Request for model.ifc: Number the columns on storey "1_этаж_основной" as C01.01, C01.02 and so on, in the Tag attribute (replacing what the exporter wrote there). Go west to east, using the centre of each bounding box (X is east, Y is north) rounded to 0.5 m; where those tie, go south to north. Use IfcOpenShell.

First a look at what the model holds.

```python
import ifcopenshell
import ifcopenshell.util.element
import ifcopenshell.util.placement

model = ifcopenshell.open("model.ifc")
print(model.schema)
storey = next(s for s in model.by_type("IfcBuildingStorey") if s.Name == "1_этаж_основной")
columns = [e for e in ifcopenshell.util.element.get_decomposition(storey) if e.is_a("IfcColumn")]
for e in sorted(columns, key=lambda e: e.id()):
    origin = ifcopenshell.util.placement.get_local_placement(e.ObjectPlacement)[:3, 3]
    print(e.id(), e.Tag, e.Name, origin.round(2) + 0.0, sep=" | ")
```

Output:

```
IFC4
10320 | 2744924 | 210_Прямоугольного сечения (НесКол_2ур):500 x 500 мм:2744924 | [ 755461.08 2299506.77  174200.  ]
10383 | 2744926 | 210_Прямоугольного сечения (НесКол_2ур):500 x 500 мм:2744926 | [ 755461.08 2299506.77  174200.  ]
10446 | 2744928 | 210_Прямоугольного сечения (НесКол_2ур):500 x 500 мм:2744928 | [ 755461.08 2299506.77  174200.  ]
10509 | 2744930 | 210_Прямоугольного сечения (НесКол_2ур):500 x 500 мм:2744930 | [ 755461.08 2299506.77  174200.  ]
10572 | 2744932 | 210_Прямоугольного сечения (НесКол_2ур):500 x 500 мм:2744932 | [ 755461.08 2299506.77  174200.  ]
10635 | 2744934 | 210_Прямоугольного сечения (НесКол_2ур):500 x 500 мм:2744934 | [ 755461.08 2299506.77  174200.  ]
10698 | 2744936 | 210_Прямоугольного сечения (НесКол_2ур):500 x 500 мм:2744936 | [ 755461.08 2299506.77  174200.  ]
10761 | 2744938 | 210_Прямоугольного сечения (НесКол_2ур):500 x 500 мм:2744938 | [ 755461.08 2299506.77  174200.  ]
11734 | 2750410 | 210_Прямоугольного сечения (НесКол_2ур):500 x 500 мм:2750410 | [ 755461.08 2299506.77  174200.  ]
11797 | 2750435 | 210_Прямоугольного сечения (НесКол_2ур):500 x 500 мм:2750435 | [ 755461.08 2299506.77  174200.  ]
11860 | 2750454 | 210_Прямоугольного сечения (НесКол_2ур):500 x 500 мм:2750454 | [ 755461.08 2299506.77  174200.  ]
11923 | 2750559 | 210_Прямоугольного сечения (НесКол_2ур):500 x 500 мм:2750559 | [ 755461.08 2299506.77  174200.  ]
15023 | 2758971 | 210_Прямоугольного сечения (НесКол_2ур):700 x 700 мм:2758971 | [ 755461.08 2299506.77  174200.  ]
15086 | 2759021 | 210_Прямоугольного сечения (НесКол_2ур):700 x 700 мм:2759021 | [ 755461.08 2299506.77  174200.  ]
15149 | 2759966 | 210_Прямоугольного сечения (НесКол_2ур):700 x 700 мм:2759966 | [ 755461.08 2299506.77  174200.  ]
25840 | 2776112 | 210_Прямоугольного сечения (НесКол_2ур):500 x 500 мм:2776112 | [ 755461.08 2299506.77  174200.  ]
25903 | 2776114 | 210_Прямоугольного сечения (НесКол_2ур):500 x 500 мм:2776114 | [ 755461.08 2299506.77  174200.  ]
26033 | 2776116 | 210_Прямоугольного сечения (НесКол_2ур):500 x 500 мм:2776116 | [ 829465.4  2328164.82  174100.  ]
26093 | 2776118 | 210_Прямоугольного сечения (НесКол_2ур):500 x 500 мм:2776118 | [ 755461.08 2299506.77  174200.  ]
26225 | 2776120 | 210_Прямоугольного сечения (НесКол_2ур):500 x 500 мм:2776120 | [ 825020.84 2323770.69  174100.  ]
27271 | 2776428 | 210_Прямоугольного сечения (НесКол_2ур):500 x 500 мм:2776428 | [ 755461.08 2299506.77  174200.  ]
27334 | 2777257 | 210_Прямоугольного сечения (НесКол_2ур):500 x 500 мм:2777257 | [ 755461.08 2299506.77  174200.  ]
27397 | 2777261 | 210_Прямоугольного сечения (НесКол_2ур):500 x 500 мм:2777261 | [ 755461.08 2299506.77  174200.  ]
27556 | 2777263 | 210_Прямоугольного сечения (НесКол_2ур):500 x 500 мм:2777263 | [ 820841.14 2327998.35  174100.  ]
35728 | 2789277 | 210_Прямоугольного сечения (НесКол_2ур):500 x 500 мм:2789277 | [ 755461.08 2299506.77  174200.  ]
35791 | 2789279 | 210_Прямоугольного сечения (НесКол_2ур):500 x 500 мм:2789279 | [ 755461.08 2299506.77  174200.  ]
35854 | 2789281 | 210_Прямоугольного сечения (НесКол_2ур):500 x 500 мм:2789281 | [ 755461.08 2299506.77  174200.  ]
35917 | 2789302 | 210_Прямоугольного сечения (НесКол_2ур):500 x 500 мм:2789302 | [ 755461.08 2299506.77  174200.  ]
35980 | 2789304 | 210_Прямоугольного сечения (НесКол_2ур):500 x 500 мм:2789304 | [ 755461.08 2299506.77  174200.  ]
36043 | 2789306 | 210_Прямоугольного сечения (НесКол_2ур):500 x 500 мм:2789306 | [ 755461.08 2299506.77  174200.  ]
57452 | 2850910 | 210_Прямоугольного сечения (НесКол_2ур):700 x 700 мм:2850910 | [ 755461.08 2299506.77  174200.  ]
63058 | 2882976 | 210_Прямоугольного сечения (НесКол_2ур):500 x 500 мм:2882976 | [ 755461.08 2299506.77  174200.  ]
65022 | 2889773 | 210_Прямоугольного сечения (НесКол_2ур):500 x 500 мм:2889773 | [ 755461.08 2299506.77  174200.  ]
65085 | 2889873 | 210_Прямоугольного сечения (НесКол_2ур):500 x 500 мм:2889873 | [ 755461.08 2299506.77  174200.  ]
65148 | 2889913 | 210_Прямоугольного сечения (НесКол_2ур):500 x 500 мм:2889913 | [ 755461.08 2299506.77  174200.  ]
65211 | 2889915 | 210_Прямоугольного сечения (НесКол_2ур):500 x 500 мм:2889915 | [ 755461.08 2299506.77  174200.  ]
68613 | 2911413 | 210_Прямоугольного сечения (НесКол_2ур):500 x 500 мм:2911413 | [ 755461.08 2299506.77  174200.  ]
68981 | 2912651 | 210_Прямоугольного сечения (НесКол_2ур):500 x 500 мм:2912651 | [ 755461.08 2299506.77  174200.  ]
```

```python
import ifcopenshell
import ifcopenshell.geom
import ifcopenshell.util.element
import ifcopenshell.util.shape

model = ifcopenshell.open("model.ifc")
settings = ifcopenshell.geom.settings()
settings.set("use-world-coords", True)


def centre(element):
    shape = ifcopenshell.geom.create_shape(settings, element)
    return ifcopenshell.util.shape.get_bbox_centroid(shape.geometry)


storey = next(s for s in model.by_type("IfcBuildingStorey") if s.Name == "1_этаж_основной")
columns = [e for e in ifcopenshell.util.element.get_decomposition(storey) if e.is_a("IfcColumn")]

# Insertion points can sit at a corner or the storey origin, so sort by the geometry (in metres).
centres = {e: centre(e) for e in columns}
columns.sort(key=lambda e: (round(centres[e][0] / 0.5), centres[e][1]))

for i, e in enumerate(columns, start=1):
    number = f"C01.{i:02d}"
    e.Tag = number
    print(e.id(), number)

model.write("model_edited.ifc")
```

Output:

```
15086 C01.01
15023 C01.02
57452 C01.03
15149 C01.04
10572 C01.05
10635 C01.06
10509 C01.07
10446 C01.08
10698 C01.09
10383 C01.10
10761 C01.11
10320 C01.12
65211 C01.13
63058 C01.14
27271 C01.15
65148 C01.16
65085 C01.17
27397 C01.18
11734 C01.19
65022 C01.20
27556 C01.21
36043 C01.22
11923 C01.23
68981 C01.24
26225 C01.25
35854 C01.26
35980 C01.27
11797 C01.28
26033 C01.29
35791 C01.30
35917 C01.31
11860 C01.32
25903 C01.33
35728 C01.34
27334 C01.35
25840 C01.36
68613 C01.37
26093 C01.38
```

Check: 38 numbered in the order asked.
